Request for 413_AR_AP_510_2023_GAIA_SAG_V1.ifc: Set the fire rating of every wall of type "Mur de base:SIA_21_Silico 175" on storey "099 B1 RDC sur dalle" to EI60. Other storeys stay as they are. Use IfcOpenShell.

First a look at what the model holds.

```python
import ifcopenshell
import ifcopenshell.util.element

model = ifcopenshell.open("413_AR_AP_510_2023_GAIA_SAG_V1.ifc")
print(model.schema)
storey = next(s for s in model.by_type("IfcBuildingStorey") if s.Name == "099 B1 RDC sur dalle")
walls = [e for e in ifcopenshell.util.element.get_decomposition(storey) if e.is_a("IfcWall")]
seen = {}
for e in walls:
    element_type = ifcopenshell.util.element.get_type(e)
    key = (element_type.Name if element_type != e and element_type else None, ifcopenshell.util.element.get_pset(e, "Pset_WallCommon", "FireRating"))
    seen[key] = seen.get(key, 0) + 1
for (name, value), count in sorted(seen.items(), key=str):
    print(count, "x", name, "|", value)
```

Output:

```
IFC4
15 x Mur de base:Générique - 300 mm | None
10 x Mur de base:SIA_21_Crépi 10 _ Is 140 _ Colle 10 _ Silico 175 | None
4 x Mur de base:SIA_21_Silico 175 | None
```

```python
import ifcopenshell
import ifcopenshell.api.pset
import ifcopenshell.util.element

model = ifcopenshell.open("413_AR_AP_510_2023_GAIA_SAG_V1.ifc")

storey = next(s for s in model.by_type("IfcBuildingStorey") if s.Name == "099 B1 RDC sur dalle")
walls = [e for e in ifcopenshell.util.element.get_decomposition(storey) if e.is_a("IfcWall")]

count = 0
for e in walls:
    element_type = ifcopenshell.util.element.get_type(e)
    if element_type in (None, e) or element_type.Name != "Mur de base:SIA_21_Silico 175":
        continue
    # add_pset returns the element's existing set when there is one.
    pset = ifcopenshell.api.pset.add_pset(model, product=e, name="Pset_WallCommon")
    ifcopenshell.api.pset.edit_pset(model, pset=pset, properties={"FireRating": "EI60"})
    count += 1

print(count, "walls updated")

model.write("413_AR_AP_510_2023_GAIA_SAG_V1_rev.ifc")
```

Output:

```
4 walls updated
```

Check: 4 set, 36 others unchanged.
